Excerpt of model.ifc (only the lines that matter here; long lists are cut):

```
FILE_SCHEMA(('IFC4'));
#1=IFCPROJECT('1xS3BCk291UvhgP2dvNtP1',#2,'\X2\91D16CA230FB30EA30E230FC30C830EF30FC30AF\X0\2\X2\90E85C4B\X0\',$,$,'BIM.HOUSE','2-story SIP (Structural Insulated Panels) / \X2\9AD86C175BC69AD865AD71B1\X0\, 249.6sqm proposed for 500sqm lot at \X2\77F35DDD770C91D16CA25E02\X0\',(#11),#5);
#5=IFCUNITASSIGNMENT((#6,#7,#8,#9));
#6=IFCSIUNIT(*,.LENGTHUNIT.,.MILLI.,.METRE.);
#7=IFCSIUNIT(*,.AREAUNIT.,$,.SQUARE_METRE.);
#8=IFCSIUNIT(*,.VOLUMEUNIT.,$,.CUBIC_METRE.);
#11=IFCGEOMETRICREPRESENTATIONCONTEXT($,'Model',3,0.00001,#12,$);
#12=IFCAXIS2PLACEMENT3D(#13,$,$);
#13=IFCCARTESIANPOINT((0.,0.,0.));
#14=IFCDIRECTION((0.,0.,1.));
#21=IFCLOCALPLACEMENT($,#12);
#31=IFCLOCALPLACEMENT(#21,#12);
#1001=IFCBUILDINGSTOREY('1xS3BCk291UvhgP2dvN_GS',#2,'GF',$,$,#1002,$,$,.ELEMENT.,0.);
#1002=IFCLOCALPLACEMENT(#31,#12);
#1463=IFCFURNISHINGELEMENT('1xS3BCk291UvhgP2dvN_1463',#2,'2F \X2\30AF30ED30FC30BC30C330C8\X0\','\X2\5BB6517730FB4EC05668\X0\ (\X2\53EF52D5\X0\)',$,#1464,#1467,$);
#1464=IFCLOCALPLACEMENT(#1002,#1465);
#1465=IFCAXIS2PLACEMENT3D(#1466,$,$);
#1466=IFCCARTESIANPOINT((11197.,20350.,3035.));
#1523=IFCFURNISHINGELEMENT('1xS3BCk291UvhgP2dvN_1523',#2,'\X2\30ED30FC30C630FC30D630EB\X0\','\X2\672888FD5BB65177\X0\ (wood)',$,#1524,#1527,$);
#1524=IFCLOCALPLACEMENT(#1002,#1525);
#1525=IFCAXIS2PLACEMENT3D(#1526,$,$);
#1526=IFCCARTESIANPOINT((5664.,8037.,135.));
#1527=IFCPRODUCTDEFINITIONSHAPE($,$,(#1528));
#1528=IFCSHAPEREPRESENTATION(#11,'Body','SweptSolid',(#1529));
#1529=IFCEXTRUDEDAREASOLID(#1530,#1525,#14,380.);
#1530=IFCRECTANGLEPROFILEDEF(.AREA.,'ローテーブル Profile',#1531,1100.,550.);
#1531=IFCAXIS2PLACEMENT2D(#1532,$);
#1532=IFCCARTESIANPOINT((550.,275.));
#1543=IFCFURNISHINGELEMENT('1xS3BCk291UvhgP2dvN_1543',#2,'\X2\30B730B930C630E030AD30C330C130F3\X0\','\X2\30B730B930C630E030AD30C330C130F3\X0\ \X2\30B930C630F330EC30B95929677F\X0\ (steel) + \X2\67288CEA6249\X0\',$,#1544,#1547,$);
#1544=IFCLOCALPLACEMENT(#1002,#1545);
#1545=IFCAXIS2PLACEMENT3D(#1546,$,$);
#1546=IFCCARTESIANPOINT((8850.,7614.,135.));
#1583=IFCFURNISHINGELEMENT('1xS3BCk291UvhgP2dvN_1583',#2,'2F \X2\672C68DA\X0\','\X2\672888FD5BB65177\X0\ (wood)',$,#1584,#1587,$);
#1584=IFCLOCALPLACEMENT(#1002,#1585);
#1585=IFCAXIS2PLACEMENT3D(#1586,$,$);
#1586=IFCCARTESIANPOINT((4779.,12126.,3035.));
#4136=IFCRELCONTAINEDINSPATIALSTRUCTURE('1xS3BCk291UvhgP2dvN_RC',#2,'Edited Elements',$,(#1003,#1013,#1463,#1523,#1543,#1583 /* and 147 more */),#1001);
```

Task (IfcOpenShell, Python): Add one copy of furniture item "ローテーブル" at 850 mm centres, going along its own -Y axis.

```python
import ifcopenshell
import ifcopenshell.api.geometry
import ifcopenshell.api.root
import ifcopenshell.util.element
import ifcopenshell.util.placement
import ifcopenshell.util.unit

model = ifcopenshell.open("model.ifc")
unit_scale = ifcopenshell.util.unit.calculate_unit_scale(model)


def reuse_history(source, copy):
    """copy_class also copies each property set's owner history, people and application; keep the originals."""
    for rel in copy.IsDefinedBy:
        if rel.is_a("IfcRelDefinesByProperties") and (history := rel.RelatingPropertyDefinition.OwnerHistory):
            rel.RelatingPropertyDefinition.OwnerHistory = source.OwnerHistory
            ifcopenshell.util.element.remove_deep2(model, history)


source = model.by_guid("1xS3BCk291UvhgP2dvN_1523")
base = ifcopenshell.util.placement.get_local_placement(source.ObjectPlacement)
step = -base[:3, 1] * 0.85 / unit_scale

for i in range(1, 2):
    copy = ifcopenshell.api.root.copy_class(model, product=source)
    copy.Representation = ifcopenshell.util.element.copy_deep(
        model, source.Representation, exclude=["IfcGeometricRepresentationContext", "IfcRepresentationMap"]
    )
    reuse_history(source, copy)
    matrix = base.copy()
    matrix[:3, 3] += i * step
    print("added at", matrix[:3, 3].round(3) + 0.0)
    ifcopenshell.api.geometry.edit_object_placement(model, product=copy, matrix=matrix, is_si=False)

model.write("model_rev.ifc")
```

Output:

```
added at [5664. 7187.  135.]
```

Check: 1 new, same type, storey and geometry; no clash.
